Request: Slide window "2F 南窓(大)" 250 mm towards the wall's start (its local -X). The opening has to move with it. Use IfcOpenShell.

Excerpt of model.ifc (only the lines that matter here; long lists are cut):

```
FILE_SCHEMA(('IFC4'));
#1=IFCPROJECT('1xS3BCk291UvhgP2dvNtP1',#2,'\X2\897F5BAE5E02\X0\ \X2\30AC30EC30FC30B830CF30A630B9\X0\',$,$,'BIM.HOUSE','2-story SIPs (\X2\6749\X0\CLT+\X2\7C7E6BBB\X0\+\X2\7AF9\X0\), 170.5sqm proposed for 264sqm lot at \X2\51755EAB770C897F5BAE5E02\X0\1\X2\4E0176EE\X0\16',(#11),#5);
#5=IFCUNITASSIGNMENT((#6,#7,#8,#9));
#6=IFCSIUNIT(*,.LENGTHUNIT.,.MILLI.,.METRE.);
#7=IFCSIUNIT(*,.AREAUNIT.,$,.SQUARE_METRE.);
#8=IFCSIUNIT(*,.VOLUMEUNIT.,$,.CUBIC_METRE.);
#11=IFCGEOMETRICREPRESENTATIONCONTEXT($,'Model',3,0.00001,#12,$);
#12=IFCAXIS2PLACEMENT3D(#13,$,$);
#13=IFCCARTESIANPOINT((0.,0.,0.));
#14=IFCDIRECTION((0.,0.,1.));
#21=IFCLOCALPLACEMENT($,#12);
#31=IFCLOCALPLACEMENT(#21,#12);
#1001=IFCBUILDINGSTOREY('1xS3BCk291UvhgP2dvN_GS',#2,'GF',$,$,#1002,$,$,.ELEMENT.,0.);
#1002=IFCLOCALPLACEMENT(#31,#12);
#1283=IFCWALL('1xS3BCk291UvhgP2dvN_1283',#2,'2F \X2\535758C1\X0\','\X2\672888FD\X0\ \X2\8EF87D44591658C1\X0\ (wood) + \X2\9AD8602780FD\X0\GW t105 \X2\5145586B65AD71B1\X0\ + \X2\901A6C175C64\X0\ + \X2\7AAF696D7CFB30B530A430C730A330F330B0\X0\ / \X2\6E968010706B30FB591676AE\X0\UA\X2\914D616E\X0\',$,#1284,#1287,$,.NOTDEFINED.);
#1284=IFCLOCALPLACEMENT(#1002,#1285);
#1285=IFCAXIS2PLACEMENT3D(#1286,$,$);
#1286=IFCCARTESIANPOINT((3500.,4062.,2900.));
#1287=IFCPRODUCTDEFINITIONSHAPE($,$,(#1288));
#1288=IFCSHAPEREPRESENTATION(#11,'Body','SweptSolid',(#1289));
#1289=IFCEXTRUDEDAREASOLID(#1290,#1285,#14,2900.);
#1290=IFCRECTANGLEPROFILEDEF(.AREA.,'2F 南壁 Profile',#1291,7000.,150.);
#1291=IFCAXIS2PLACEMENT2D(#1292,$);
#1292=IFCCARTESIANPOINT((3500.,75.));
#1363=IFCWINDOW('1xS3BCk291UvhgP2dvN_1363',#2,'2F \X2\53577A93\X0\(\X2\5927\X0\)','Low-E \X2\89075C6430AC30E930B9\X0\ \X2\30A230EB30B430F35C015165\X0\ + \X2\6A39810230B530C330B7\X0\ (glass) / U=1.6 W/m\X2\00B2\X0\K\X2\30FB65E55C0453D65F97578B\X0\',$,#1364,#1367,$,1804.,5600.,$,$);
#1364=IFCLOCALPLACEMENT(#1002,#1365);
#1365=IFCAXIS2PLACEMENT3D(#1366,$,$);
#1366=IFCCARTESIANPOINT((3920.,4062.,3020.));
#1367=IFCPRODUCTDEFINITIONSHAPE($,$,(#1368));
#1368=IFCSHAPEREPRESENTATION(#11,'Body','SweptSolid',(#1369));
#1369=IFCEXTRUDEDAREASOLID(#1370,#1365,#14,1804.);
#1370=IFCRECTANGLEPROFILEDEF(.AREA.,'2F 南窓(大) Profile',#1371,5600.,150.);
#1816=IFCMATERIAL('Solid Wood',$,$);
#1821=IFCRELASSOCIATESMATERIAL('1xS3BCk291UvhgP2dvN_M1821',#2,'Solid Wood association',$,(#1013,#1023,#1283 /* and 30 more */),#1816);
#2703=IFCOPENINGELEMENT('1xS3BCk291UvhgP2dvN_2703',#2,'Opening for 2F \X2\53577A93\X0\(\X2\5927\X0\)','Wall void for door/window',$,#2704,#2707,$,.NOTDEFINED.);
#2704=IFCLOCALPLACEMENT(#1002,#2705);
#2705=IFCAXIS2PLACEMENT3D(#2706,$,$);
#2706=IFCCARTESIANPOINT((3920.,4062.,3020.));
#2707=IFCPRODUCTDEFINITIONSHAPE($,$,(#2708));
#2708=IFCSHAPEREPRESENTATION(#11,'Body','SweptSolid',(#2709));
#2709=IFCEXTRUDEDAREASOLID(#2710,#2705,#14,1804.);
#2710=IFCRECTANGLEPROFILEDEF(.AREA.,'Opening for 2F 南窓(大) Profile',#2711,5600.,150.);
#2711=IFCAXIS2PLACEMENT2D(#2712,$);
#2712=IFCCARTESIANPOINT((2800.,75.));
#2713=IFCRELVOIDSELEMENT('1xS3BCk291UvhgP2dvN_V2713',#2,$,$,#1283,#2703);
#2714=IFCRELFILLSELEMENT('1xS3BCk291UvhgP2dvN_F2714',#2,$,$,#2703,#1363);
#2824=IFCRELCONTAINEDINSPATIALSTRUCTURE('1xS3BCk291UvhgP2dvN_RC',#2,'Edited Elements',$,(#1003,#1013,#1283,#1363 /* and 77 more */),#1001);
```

```python
import ifcopenshell
import ifcopenshell.api.geometry
import ifcopenshell.util.placement
import ifcopenshell.util.unit

model = ifcopenshell.open("model.ifc")
unit_scale = ifcopenshell.util.unit.calculate_unit_scale(model)

window = model.by_guid("1xS3BCk291UvhgP2dvN_1363")
opening = window.FillsVoids[0].RelatingOpeningElement
wall = opening.VoidsElements[0].RelatingBuildingElement

wall_matrix = ifcopenshell.util.placement.get_local_placement(wall.ObjectPlacement)
shift = wall_matrix[:3, 0] * -0.25 / unit_scale
before = ifcopenshell.util.placement.get_local_placement(window.ObjectPlacement)[:3, 3].copy()

# The window is not placed relative to its opening, so move both.
for product in (opening, window):
    matrix = ifcopenshell.util.placement.get_local_placement(product.ObjectPlacement)
    matrix[:3, 3] += shift
    ifcopenshell.api.geometry.edit_object_placement(model, product=product, matrix=matrix, is_si=False)

after = ifcopenshell.util.placement.get_local_placement(window.ObjectPlacement)[:3, 3]
print("window moved by", (after - before).round(3) + 0.0)

model.write("model_updated.ifc")
```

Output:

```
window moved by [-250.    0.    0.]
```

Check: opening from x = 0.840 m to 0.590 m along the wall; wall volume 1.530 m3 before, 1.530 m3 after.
